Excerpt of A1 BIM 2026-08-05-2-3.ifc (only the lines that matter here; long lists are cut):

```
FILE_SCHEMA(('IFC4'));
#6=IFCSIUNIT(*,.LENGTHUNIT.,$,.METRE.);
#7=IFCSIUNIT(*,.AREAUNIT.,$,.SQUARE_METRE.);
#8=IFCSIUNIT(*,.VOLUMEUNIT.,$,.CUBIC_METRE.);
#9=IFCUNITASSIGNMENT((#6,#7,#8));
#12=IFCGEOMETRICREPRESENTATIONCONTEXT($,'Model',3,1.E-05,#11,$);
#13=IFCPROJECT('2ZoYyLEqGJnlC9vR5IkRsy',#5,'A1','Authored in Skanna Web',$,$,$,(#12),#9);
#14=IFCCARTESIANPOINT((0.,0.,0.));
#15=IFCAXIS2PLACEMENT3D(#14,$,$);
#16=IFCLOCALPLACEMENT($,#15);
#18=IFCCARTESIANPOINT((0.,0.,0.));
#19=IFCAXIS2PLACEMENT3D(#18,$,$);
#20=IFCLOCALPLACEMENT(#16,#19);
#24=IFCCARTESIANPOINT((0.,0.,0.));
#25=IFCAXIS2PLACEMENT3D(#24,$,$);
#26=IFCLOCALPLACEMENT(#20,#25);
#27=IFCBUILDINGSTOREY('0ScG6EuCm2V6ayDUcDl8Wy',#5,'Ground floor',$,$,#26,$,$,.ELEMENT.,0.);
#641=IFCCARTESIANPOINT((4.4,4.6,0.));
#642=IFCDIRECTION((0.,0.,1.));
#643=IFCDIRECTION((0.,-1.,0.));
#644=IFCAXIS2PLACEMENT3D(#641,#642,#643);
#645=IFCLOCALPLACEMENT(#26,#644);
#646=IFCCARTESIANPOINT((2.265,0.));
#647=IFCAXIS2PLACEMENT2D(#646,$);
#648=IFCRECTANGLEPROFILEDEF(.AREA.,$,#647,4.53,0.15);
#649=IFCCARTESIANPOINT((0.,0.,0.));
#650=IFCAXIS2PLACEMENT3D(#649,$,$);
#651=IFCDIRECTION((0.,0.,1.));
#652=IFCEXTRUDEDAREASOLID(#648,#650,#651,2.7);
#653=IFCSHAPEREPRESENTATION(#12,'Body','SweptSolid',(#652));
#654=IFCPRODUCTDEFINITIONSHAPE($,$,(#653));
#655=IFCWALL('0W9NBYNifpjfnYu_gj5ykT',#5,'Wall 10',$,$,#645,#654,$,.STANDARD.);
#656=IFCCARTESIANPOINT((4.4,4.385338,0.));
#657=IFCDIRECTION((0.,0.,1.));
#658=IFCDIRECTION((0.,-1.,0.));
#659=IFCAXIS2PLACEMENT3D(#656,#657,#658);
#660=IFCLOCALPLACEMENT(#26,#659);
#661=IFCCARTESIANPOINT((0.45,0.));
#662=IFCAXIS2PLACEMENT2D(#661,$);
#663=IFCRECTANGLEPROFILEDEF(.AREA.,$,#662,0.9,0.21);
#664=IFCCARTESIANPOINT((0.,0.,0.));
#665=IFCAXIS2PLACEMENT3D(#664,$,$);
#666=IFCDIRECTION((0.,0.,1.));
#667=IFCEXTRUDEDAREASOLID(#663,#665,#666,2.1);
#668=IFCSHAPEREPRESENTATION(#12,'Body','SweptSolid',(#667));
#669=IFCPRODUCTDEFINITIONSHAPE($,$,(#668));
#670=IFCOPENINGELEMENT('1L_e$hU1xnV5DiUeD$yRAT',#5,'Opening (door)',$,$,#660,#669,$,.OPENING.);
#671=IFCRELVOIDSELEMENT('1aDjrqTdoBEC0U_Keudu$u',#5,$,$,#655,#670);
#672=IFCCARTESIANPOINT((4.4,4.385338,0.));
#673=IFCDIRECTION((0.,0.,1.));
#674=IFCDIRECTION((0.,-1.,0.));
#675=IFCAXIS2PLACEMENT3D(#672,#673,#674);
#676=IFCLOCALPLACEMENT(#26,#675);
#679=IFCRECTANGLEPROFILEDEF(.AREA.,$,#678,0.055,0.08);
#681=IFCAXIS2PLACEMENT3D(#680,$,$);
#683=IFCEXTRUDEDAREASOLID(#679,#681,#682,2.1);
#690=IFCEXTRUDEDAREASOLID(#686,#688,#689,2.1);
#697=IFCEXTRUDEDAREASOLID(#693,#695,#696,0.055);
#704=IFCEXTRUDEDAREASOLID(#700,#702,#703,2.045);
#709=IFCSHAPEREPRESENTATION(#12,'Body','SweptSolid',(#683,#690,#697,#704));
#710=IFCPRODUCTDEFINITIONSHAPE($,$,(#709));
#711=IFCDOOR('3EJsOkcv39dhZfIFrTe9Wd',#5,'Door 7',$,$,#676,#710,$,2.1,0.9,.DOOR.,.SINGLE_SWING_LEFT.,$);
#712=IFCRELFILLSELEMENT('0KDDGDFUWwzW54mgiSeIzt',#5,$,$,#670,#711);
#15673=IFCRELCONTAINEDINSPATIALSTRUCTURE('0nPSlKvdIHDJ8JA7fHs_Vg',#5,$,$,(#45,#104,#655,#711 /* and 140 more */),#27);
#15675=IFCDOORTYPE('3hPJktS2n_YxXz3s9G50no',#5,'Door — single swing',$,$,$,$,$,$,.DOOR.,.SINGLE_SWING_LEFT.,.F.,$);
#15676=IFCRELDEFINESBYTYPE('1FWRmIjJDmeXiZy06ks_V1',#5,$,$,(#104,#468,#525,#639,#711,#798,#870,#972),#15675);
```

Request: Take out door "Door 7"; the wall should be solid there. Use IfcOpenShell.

```python
import ifcopenshell
import ifcopenshell.api.feature
import ifcopenshell.api.root
import ifcopenshell.geom
import ifcopenshell.util.shape

model = ifcopenshell.open("A1 BIM 2026-08-05-2-3.ifc")
settings = ifcopenshell.geom.settings()


def volume(element):
    """Net volume in cubic metres, openings subtracted."""
    shape = ifcopenshell.geom.create_shape(settings, element)
    return ifcopenshell.util.shape.get_volume(shape.geometry)


door = model.by_guid("3EJsOkcv39dhZfIFrTe9Wd")
opening = door.FillsVoids[0].RelatingOpeningElement
wall = opening.VoidsElements[0].RelatingBuildingElement
before = volume(wall)

ifcopenshell.api.root.remove_product(model, product=door)
ifcopenshell.api.feature.remove_feature(model, feature=opening)

after = volume(wall)

print(f"wall volume {before:.3f} -> {after:.3f} m3")

model.write("A1 BIM 2026-08-05-2-3_edited.ifc")
```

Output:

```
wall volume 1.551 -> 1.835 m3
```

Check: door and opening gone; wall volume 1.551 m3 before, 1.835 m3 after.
